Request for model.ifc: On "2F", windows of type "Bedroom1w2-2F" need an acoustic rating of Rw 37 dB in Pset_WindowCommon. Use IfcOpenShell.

First a look at what the model holds.

```python
import ifcopenshell
import ifcopenshell.util.element

model = ifcopenshell.open("model.ifc")
print(model.schema)
storey = next(s for s in model.by_type("IfcBuildingStorey") if s.Name == "2F")
windows = [e for e in ifcopenshell.util.element.get_decomposition(storey) if e.is_a("IfcWindow")]
seen = {}
for e in windows:
    element_type = ifcopenshell.util.element.get_type(e)
    key = (element_type.Name if element_type != e and element_type else None, ifcopenshell.util.element.get_pset(e, "Pset_WindowCommon", "AcousticRating"))
    seen[key] = seen.get(key, 0) + 1
for (name, value), count in sorted(seen.items(), key=str):
    print(count, "x", name, "|", value)
```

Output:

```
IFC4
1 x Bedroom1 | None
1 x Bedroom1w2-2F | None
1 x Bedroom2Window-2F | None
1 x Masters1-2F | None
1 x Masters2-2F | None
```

```python
import ifcopenshell
import ifcopenshell.api.pset
import ifcopenshell.util.element

model = ifcopenshell.open("model.ifc")

storey = next(s for s in model.by_type("IfcBuildingStorey") if s.Name == "2F")
windows = [e for e in ifcopenshell.util.element.get_decomposition(storey) if e.is_a("IfcWindow")]

count = 0
for e in windows:
    element_type = ifcopenshell.util.element.get_type(e)
    if element_type in (None, e) or element_type.Name != "Bedroom1w2-2F":
        continue
    # add_pset returns the element's existing set when there is one.
    pset = ifcopenshell.api.pset.add_pset(model, product=e, name="Pset_WindowCommon")
    ifcopenshell.api.pset.edit_pset(model, pset=pset, properties={"AcousticRating": "Rw 37 dB"})
    count += 1

print(count, "windows updated")

model.write("model-out.ifc")
```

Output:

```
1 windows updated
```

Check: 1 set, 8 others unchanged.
